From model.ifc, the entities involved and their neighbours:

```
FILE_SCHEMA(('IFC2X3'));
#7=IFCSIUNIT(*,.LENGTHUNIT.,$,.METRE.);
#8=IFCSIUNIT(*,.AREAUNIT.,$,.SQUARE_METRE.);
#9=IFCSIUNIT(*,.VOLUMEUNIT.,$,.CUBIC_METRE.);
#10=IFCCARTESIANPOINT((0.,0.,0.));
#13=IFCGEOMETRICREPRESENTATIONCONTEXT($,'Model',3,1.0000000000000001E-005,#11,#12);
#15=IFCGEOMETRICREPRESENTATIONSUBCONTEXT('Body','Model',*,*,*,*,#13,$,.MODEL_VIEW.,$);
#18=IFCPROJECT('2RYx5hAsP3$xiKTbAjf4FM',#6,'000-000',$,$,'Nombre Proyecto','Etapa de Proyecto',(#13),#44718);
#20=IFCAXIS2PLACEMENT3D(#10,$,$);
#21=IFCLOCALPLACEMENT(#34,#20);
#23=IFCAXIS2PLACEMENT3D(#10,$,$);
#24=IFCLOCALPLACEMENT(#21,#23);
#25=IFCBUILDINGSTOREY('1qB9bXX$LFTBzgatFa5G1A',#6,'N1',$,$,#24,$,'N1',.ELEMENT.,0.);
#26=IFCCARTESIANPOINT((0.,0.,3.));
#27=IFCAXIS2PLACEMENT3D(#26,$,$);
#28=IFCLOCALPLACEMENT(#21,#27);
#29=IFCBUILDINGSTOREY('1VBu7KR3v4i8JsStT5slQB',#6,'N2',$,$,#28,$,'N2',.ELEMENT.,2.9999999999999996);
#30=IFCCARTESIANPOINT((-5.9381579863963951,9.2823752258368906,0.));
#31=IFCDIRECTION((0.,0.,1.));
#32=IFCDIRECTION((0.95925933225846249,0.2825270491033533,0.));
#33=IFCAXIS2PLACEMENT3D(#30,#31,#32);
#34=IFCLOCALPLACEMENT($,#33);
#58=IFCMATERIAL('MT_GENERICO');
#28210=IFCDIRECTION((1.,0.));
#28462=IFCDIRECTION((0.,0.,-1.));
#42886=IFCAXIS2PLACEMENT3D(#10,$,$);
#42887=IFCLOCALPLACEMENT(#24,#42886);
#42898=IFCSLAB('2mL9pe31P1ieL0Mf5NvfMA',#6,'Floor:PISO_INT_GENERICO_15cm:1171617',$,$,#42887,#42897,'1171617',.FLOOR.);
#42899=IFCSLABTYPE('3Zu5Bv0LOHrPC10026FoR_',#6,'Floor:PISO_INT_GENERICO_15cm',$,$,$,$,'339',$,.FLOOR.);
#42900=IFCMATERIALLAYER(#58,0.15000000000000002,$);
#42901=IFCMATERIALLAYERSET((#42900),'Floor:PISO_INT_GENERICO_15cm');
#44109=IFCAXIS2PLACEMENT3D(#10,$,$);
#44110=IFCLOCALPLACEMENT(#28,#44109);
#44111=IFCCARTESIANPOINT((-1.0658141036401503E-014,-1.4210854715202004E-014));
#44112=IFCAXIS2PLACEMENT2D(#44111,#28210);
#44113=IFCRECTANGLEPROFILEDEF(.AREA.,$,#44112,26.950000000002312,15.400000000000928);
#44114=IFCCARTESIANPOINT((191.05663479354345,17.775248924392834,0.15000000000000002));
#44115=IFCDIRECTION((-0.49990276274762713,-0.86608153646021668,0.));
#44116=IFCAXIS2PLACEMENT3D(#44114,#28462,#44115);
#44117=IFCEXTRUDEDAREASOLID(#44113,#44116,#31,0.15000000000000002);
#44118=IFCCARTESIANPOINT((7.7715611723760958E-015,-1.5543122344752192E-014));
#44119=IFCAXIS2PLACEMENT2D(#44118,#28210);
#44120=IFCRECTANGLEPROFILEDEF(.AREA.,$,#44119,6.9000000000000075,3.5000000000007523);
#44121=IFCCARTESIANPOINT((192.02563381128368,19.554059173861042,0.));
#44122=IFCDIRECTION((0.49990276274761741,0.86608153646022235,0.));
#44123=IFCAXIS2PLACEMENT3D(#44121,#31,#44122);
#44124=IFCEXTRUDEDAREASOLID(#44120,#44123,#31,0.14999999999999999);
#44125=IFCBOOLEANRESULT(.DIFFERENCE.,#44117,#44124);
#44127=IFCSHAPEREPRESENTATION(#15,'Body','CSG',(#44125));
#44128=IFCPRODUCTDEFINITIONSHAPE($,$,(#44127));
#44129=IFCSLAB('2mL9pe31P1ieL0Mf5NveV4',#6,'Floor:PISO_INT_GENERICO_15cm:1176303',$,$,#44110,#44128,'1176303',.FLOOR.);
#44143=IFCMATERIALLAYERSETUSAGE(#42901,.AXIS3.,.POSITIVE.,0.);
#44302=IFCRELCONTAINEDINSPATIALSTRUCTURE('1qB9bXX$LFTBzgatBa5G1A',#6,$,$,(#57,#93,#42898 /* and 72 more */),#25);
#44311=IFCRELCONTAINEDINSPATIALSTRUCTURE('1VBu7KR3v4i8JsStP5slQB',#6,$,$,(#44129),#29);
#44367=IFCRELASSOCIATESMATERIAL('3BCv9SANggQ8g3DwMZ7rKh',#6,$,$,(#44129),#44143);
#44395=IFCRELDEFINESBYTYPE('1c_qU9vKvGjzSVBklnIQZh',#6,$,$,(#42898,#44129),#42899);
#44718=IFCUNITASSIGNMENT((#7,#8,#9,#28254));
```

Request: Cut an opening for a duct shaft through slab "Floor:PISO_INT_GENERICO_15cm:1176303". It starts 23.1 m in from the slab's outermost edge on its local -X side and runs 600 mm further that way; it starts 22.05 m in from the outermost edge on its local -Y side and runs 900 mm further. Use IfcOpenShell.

```python
import numpy as np
import ifcopenshell
import ifcopenshell.api.feature
import ifcopenshell.api.geometry
import ifcopenshell.api.root
import ifcopenshell.geom
import ifcopenshell.util.placement
import ifcopenshell.util.representation
import ifcopenshell.util.shape
import ifcopenshell.util.unit

model = ifcopenshell.open("model.ifc")
unit_scale = ifcopenshell.util.unit.calculate_unit_scale(model)
settings = ifcopenshell.geom.settings()


def volume(element):
    """Net volume in cubic metres, openings subtracted."""
    shape = ifcopenshell.geom.create_shape(settings, element)
    return ifcopenshell.util.shape.get_volume(shape.geometry)


slab = model.by_guid("2mL9pe31P1ieL0Mf5NveV4")
before = volume(slab)

# Extent in the slab's own axes, in metres. The edges named are its -X and -Y sides.
slab_shape = ifcopenshell.geom.create_shape(settings, slab)
vertices = ifcopenshell.util.shape.get_vertices(slab_shape.geometry)
x_min, y_min, bottom = vertices.min(axis=0)
top = vertices[:, 2].max()

opening = ifcopenshell.api.root.create_entity(model, ifc_class="IfcOpeningElement", name="Duct shaft opening")
context = ifcopenshell.util.representation.get_context(model, "Model", "Body", "MODEL_VIEW")
width, depth = 0.6, 0.9
outline = [(0.0, 0.0), (width, 0.0), (width, depth), (0.0, depth), (0.0, 0.0)]
# Overshoot both faces by 50 mm so the cut is clean.
shape = ifcopenshell.api.geometry.add_slab_representation(
    model, context=context, depth=top - bottom + 0.1, polyline=outline
)
ifcopenshell.api.geometry.assign_representation(model, product=opening, representation=shape)

matrix = ifcopenshell.util.placement.get_local_placement(slab.ObjectPlacement)
matrix[:, 3] = matrix @ np.append(np.array([x_min + 23.1, y_min + 22.05, bottom - 0.05]) / unit_scale, 1.0)
ifcopenshell.api.geometry.edit_object_placement(model, product=opening, matrix=matrix, is_si=False)
ifcopenshell.api.feature.add_feature(model, feature=opening, element=slab)

after = volume(slab)

print(f"slab volume {before:.3f} -> {after:.3f} m3")

model.write("model_v2.ifc")
```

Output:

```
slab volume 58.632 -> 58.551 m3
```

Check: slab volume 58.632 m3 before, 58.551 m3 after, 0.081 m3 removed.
